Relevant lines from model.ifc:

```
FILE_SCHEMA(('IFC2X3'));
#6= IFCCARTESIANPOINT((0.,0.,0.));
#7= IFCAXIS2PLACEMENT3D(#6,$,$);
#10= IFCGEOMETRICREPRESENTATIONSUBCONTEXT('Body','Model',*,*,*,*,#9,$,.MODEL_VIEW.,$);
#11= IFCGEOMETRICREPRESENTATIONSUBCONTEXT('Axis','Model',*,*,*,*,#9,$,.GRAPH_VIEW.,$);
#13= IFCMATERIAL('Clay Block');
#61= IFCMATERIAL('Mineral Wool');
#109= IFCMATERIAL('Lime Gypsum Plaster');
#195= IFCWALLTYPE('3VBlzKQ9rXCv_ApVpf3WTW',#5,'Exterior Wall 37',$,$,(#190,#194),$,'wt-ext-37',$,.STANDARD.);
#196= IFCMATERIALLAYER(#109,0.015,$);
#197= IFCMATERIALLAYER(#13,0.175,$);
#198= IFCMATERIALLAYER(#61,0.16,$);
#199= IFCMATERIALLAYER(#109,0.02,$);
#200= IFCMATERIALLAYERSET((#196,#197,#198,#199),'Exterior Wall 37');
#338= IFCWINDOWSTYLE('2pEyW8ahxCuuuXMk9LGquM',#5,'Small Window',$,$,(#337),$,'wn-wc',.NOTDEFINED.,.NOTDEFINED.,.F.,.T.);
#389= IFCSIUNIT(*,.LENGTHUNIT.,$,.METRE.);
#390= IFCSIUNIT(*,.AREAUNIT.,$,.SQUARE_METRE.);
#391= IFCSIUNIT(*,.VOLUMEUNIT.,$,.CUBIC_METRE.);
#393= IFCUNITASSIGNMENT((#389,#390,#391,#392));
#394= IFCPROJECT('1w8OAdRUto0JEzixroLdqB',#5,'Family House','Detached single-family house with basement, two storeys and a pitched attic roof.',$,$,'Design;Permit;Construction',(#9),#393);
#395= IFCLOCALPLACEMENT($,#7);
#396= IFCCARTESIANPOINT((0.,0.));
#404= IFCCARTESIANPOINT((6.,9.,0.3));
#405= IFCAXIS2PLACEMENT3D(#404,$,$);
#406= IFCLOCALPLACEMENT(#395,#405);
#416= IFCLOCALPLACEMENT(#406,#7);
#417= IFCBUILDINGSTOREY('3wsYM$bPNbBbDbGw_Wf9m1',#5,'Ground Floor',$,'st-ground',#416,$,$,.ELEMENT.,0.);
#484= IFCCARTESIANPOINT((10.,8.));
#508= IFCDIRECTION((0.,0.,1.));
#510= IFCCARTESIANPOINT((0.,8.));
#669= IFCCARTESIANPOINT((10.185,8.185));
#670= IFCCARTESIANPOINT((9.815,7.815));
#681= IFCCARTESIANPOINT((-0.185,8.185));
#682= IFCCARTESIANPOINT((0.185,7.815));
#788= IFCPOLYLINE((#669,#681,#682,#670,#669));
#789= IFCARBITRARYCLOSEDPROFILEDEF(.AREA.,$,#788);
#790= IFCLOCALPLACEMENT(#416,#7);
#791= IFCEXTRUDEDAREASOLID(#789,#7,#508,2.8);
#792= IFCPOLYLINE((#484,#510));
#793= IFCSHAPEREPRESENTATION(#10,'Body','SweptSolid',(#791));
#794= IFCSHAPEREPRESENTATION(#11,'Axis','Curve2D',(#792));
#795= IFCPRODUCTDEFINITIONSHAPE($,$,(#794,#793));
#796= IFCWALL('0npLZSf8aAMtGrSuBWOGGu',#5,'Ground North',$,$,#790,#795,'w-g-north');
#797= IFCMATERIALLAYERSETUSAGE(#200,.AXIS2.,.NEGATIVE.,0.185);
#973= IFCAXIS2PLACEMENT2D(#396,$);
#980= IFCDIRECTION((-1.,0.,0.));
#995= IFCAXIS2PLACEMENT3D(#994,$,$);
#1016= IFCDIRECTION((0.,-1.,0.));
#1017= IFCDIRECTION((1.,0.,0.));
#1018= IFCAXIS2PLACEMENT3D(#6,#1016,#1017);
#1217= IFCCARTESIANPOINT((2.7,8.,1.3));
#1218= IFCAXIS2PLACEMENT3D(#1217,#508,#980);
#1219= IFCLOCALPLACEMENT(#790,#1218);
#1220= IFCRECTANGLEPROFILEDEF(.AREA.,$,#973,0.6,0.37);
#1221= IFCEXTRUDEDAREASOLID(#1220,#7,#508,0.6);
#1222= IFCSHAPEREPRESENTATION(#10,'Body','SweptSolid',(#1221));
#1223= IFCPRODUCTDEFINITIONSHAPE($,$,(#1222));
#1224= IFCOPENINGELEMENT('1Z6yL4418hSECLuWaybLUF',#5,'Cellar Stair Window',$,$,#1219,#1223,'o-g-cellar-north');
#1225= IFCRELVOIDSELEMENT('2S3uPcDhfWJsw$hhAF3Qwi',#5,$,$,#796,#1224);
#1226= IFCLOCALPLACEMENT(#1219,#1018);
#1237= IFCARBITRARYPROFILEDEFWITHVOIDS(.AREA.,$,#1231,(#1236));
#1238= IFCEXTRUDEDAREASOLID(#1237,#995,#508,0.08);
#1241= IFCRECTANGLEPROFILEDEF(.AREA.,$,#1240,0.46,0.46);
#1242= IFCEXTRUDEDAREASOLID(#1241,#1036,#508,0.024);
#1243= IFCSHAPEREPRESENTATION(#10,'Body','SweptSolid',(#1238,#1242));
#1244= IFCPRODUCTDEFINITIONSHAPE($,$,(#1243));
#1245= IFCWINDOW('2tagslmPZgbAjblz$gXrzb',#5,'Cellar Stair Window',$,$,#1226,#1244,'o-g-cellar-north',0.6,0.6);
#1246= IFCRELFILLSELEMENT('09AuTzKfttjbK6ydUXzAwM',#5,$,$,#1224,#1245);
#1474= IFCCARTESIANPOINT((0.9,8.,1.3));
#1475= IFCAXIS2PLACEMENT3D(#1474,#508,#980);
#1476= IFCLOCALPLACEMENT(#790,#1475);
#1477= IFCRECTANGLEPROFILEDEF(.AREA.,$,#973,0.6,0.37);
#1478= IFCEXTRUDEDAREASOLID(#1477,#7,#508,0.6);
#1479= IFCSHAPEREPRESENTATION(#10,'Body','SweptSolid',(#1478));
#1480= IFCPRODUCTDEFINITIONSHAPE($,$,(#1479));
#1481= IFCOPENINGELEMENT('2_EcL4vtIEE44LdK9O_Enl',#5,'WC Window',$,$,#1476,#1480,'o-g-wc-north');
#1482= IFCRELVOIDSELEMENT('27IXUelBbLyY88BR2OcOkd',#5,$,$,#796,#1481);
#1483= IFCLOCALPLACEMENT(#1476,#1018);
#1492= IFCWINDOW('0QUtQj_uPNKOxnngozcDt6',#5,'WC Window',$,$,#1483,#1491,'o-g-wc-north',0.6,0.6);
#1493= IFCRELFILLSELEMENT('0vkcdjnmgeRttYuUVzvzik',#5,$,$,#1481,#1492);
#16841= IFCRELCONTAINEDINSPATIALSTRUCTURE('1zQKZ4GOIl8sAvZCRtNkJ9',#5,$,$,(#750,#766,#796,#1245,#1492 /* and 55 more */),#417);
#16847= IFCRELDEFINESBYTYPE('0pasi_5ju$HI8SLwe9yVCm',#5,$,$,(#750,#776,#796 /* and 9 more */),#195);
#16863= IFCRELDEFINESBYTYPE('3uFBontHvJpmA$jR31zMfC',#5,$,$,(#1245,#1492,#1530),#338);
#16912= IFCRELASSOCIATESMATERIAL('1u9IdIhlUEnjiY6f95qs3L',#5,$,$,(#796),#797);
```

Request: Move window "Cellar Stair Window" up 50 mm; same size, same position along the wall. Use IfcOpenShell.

```python
import numpy as np
import ifcopenshell
import ifcopenshell.api.geometry
import ifcopenshell.util.placement
import ifcopenshell.util.unit

model = ifcopenshell.open("model.ifc")
unit_scale = ifcopenshell.util.unit.calculate_unit_scale(model)

window = model.by_guid("2tagslmPZgbAjblz$gXrzb")
opening = window.FillsVoids[0].RelatingOpeningElement
dz = 0.05 / unit_scale

shift = np.array([0.0, 0.0, dz])
# The window is placed relative to its opening, so it follows when the opening moves.
matrix = ifcopenshell.util.placement.get_local_placement(opening.ObjectPlacement)
matrix[:3, 3] += shift
ifcopenshell.api.geometry.edit_object_placement(
    model, product=opening, matrix=matrix, is_si=False, should_transform_children=True
)

print(f"moved by {dz * unit_scale:+.3f} m")

model.write("model_updated.ifc")
```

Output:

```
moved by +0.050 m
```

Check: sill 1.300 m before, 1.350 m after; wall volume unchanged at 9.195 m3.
